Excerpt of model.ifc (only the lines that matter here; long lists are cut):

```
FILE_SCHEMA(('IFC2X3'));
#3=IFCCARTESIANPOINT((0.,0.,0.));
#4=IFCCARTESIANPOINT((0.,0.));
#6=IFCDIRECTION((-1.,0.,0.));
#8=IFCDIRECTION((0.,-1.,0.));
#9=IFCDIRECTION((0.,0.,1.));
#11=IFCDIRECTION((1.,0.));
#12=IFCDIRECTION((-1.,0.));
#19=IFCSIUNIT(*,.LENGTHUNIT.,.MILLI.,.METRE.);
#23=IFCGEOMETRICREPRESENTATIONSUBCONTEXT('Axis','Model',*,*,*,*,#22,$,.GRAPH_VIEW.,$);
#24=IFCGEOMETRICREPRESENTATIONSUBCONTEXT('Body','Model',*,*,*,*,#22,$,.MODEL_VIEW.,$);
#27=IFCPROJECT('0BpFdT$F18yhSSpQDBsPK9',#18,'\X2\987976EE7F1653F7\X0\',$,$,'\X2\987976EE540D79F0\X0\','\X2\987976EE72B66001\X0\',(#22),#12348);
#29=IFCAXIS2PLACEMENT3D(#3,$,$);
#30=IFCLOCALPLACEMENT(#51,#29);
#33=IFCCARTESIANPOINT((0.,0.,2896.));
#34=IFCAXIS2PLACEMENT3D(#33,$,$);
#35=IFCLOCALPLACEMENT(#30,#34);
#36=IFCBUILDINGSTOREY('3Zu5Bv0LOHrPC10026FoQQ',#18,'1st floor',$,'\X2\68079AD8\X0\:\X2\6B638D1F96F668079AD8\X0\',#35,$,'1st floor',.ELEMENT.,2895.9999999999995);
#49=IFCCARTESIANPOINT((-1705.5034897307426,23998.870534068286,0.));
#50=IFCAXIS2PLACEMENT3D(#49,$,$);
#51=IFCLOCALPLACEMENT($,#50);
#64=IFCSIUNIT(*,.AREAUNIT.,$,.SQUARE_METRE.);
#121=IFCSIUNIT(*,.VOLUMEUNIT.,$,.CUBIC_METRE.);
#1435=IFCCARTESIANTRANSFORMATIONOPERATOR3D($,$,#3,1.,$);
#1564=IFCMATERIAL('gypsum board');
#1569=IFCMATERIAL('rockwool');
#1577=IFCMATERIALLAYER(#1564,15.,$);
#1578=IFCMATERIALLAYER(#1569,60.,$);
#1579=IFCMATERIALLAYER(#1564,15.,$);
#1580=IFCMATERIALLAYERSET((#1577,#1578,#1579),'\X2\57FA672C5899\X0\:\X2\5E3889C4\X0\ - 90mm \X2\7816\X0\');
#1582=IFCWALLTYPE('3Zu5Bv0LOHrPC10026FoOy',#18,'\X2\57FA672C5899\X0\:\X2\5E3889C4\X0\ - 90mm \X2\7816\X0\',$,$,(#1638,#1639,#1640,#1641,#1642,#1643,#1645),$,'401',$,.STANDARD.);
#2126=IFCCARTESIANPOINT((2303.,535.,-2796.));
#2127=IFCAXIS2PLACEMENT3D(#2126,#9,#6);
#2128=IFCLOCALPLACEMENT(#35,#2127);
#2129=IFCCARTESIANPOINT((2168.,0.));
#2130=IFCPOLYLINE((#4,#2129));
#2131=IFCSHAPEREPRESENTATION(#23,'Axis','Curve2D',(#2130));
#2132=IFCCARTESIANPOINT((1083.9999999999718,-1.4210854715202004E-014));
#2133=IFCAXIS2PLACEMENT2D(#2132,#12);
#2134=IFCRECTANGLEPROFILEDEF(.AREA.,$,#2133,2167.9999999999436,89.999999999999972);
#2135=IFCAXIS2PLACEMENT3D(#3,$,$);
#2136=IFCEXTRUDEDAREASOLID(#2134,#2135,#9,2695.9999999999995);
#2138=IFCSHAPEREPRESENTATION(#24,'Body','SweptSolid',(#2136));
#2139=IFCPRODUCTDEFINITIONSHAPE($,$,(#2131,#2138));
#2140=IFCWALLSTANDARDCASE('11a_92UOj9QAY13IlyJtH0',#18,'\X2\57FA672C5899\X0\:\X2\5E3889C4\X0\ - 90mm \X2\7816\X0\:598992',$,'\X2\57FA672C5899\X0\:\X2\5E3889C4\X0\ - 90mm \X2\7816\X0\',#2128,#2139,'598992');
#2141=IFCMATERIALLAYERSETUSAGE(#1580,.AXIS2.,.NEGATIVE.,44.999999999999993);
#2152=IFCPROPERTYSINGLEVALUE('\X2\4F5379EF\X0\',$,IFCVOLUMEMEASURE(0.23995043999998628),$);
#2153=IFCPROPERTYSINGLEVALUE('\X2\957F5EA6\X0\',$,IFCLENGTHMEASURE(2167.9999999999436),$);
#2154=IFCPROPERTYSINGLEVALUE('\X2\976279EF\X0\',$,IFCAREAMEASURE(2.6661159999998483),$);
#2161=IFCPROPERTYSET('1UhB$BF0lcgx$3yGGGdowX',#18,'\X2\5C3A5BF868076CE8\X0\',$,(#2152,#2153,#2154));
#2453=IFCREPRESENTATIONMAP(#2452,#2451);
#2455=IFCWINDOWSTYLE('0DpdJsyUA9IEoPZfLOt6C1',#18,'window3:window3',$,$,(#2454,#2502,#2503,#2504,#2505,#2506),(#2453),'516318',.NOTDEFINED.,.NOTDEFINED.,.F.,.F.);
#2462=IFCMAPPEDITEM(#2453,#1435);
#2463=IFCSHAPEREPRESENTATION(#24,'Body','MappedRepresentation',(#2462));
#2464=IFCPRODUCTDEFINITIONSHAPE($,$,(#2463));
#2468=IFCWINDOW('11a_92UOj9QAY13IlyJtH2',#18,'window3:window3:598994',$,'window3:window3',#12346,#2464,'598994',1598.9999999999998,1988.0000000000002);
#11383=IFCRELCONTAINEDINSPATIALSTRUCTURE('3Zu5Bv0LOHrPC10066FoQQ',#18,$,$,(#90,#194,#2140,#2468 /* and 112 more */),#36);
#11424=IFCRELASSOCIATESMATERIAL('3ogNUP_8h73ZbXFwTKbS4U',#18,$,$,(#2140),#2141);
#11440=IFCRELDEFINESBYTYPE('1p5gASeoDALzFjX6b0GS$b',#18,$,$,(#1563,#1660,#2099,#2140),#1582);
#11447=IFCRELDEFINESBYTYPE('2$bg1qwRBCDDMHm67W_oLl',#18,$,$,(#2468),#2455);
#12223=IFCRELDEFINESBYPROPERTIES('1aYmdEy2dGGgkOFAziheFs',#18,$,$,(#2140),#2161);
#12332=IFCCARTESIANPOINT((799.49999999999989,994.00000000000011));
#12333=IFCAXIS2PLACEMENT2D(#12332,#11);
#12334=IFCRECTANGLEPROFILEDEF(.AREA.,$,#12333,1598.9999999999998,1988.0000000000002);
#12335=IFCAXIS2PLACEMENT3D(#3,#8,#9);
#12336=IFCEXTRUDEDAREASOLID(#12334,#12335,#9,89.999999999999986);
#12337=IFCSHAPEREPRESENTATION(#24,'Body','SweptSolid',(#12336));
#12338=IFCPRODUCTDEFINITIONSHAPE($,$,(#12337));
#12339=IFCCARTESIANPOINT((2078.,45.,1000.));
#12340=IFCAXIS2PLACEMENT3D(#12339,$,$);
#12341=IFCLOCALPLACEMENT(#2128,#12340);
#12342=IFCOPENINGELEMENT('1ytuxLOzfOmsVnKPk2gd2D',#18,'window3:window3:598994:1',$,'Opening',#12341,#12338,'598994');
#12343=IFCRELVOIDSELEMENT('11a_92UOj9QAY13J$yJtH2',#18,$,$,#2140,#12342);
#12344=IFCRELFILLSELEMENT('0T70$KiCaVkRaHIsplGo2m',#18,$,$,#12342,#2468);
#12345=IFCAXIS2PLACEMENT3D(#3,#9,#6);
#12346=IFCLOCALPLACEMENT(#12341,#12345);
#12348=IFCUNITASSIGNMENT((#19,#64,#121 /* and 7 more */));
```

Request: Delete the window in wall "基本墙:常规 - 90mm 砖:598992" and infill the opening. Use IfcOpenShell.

```python
import ifcopenshell
import ifcopenshell.api.feature
import ifcopenshell.api.pset
import ifcopenshell.api.root
import ifcopenshell.geom
import ifcopenshell.util.element
import ifcopenshell.util.shape
import ifcopenshell.util.unit

model = ifcopenshell.open("model.ifc")
area_scale = ifcopenshell.util.unit.calculate_unit_scale(model, "AREAUNIT")
volume_scale = ifcopenshell.util.unit.calculate_unit_scale(model, "VOLUMEUNIT")
settings = ifcopenshell.geom.settings()


def volume(element):
    """Net volume in cubic metres, openings subtracted."""
    shape = ifcopenshell.geom.create_shape(settings, element)
    return ifcopenshell.util.shape.get_volume(shape.geometry)


window = model.by_guid("11a_92UOj9QAY13IlyJtH2")
opening = window.FillsVoids[0].RelatingOpeningElement
wall = opening.VoidsElements[0].RelatingBuildingElement
before = volume(wall)

ifcopenshell.api.root.remove_product(model, product=window)
ifcopenshell.api.feature.remove_feature(model, feature=opening)

after = volume(wall)
thickness = 0.09  # wall thickness in metres

# Update the wall's stored quantities.
pset = model.by_id(ifcopenshell.util.element.get_pset(wall, "尺寸标注", should_inherit=False)["id"])
ifcopenshell.api.pset.edit_pset(model, pset=pset, properties={
    "体积": model.create_entity("IfcVolumeMeasure", after / volume_scale),
    "面积": model.create_entity("IfcAreaMeasure", after / thickness / area_scale),
})

print(f"wall volume {before:.3f} -> {after:.3f} m3")

model.write("model_edited.ifc")
```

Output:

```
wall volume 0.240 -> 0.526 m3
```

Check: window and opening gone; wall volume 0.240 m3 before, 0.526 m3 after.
